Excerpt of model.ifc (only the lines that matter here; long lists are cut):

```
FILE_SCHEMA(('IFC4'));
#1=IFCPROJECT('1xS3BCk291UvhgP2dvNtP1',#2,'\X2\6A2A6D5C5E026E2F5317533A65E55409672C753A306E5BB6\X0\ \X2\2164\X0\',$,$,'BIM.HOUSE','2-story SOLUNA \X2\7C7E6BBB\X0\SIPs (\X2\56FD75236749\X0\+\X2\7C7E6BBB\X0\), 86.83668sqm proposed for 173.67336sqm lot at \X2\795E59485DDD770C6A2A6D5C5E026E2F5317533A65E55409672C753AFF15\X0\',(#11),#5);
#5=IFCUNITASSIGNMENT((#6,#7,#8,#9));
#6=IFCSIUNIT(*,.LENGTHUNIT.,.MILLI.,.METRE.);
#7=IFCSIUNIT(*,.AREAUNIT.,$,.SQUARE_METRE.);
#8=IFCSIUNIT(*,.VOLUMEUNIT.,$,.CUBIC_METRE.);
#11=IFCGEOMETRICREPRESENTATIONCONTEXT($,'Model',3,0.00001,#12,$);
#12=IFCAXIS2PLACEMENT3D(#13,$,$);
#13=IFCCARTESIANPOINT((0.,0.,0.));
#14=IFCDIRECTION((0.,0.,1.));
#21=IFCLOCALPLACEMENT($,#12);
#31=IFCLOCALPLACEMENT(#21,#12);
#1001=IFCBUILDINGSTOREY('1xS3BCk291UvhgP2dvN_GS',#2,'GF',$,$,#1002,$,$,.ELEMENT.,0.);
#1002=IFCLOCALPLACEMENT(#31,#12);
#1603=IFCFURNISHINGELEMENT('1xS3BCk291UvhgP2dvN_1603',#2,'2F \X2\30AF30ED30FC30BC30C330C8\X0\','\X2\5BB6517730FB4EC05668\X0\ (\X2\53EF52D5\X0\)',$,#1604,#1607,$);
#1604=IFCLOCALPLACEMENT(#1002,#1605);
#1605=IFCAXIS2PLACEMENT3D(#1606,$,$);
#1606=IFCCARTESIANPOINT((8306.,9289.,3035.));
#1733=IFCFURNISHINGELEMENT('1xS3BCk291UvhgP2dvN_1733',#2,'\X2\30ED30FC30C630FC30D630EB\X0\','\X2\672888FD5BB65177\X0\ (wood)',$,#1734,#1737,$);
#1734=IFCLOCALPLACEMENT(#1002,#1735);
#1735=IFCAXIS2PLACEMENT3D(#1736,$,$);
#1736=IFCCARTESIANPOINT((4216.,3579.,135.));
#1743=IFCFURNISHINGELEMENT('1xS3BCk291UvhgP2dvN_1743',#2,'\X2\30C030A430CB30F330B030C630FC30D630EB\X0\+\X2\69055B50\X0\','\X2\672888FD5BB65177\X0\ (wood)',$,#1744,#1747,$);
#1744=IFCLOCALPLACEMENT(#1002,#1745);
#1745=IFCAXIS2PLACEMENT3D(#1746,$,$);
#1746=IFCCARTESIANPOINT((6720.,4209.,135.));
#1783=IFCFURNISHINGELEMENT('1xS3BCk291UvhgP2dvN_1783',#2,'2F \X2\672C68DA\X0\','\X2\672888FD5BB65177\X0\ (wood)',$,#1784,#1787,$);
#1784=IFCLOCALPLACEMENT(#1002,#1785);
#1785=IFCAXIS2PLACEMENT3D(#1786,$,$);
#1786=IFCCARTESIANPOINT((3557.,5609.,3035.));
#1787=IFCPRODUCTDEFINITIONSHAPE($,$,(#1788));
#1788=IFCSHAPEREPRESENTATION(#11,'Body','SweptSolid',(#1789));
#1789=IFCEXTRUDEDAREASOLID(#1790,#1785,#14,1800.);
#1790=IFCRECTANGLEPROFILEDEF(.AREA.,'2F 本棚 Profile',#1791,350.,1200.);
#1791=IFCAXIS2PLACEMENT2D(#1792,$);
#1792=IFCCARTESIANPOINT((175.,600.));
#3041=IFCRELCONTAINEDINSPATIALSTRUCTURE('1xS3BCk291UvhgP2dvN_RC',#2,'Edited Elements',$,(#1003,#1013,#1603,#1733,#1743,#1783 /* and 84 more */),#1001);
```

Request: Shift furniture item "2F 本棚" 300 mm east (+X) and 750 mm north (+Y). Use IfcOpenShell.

```python
import ifcopenshell
import ifcopenshell.api.geometry
import ifcopenshell.util.placement

model = ifcopenshell.open("model.ifc")

item = model.by_id(1783)
matrix = ifcopenshell.util.placement.get_local_placement(item.ObjectPlacement)
matrix[0, 3] += 300.0
matrix[1, 3] += 750.0
ifcopenshell.api.geometry.edit_object_placement(model, product=item, matrix=matrix, is_si=False)

print(ifcopenshell.util.placement.get_local_placement(item.ObjectPlacement).round(3) + 0.0)

model.write("model_updated.ifc")
```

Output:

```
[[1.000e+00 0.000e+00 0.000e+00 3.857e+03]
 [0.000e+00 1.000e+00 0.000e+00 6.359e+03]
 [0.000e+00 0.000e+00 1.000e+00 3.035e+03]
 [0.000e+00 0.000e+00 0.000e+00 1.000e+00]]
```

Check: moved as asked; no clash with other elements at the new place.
